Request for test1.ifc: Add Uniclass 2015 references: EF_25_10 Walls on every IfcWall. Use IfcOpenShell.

First a look at what the model holds.

```python
import ifcopenshell

model = ifcopenshell.open("test1.ifc")
print(model.schema)
print("classifications:", [c.Name for c in model.by_type("IfcClassification")])
for ifc_class in ("IfcDoor", "IfcRoof", "IfcStair", "IfcWall", "IfcWindow"):
    print(ifc_class, len(model.by_type(ifc_class)))
```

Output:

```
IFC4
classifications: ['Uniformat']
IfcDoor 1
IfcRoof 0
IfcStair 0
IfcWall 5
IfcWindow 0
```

```python
import ifcopenshell
import ifcopenshell.api.classification

model = ifcopenshell.open("test1.ifc")

system = ifcopenshell.api.classification.add_classification(model, classification="Uniclass 2015")

codes = {
    "IfcWall": ("EF_25_10", "Walls"),
}
for ifc_class, (code, name) in codes.items():
    products = model.by_type(ifc_class)
    ifcopenshell.api.classification.add_reference(
        model, products=products, classification=system, identification=code, name=name
    )
    print(code, len(products))

model.write("test1_updated.ifc")
```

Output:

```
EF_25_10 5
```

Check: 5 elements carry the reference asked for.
